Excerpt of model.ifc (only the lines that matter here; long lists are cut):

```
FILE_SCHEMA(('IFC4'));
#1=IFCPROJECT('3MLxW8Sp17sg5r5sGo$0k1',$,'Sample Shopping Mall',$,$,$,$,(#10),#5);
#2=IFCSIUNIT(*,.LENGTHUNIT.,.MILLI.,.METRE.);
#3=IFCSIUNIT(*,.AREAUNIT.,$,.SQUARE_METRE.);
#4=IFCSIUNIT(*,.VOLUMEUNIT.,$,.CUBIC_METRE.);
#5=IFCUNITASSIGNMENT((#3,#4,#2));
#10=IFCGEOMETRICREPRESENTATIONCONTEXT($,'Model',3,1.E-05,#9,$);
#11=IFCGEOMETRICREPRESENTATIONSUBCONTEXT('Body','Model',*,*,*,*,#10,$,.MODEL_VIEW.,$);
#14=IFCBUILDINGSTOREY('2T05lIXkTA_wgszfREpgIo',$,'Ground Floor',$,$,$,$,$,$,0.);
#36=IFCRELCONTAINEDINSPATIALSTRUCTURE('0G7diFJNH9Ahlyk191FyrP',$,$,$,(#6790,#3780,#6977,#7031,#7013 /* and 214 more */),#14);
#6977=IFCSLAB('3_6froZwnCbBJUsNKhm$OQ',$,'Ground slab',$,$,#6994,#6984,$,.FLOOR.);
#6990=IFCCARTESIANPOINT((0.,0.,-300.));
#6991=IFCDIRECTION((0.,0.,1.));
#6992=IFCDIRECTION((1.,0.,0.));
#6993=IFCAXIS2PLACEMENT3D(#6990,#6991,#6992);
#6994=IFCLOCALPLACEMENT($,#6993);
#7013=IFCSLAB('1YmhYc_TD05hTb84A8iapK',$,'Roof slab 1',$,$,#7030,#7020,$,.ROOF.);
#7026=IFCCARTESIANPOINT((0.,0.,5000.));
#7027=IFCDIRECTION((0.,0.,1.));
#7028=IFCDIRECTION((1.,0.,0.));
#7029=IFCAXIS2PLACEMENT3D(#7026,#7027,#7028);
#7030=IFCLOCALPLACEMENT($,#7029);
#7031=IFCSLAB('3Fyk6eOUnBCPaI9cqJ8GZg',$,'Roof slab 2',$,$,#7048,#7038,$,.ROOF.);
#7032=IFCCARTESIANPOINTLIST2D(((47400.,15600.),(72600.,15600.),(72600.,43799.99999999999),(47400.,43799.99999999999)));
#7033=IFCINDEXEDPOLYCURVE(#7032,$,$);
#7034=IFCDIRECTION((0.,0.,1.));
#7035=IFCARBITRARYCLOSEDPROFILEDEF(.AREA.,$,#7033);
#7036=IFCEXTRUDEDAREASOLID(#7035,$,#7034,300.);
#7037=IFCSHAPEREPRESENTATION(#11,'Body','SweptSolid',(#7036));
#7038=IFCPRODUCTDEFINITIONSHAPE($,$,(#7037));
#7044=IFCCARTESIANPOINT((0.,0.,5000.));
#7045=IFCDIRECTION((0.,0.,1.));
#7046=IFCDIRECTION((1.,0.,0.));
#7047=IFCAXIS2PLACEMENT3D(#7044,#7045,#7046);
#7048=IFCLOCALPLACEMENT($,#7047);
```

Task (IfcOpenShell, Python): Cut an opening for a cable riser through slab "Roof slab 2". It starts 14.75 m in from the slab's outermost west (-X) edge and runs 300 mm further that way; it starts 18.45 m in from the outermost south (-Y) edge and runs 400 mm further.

```python
import numpy as np
import ifcopenshell
import ifcopenshell.api.feature
import ifcopenshell.api.geometry
import ifcopenshell.api.root
import ifcopenshell.geom
import ifcopenshell.util.placement
import ifcopenshell.util.representation
import ifcopenshell.util.shape
import ifcopenshell.util.unit

model = ifcopenshell.open("model.ifc")
unit_scale = ifcopenshell.util.unit.calculate_unit_scale(model)
settings = ifcopenshell.geom.settings()


def volume(element):
    """Net volume in cubic metres, openings subtracted."""
    shape = ifcopenshell.geom.create_shape(settings, element)
    return ifcopenshell.util.shape.get_volume(shape.geometry)


slab = model.by_guid("3Fyk6eOUnBCPaI9cqJ8GZg")
before = volume(slab)

# Extent in the slab's own axes, in metres. The edges named are its -X and -Y sides.
slab_shape = ifcopenshell.geom.create_shape(settings, slab)
vertices = ifcopenshell.util.shape.get_vertices(slab_shape.geometry)
x_min, y_min, bottom = vertices.min(axis=0)
top = vertices[:, 2].max()

opening = ifcopenshell.api.root.create_entity(model, ifc_class="IfcOpeningElement", name="Cable riser opening", predefined_type="OPENING")
context = ifcopenshell.util.representation.get_context(model, "Model", "Body", "MODEL_VIEW")
width, depth = 0.3, 0.4
outline = [(0.0, 0.0), (width, 0.0), (width, depth), (0.0, depth), (0.0, 0.0)]
# Overshoot both faces by 50 mm so the cut is clean.
shape = ifcopenshell.api.geometry.add_slab_representation(
    model, context=context, depth=top - bottom + 0.1, polyline=outline
)
ifcopenshell.api.geometry.assign_representation(model, product=opening, representation=shape)

matrix = ifcopenshell.util.placement.get_local_placement(slab.ObjectPlacement)
matrix[:, 3] = matrix @ np.append(np.array([x_min + 14.75, y_min + 18.45, bottom - 0.05]) / unit_scale, 1.0)
ifcopenshell.api.geometry.edit_object_placement(model, product=opening, matrix=matrix, is_si=False)
ifcopenshell.api.feature.add_feature(model, feature=opening, element=slab)

after = volume(slab)

print(f"slab volume {before:.3f} -> {after:.3f} m3")

model.write("model_edited.ifc")
```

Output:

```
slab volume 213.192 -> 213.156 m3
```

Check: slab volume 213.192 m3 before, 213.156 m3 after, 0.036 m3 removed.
